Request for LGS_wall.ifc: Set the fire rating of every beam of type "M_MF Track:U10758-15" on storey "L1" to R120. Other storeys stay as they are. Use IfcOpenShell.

First a look at what the model holds.

```python
import ifcopenshell
import ifcopenshell.util.element

model = ifcopenshell.open("LGS_wall.ifc")
print(model.schema)
storey = next(s for s in model.by_type("IfcBuildingStorey") if s.Name == "L1")
beams = [e for e in ifcopenshell.util.element.get_decomposition(storey) if e.is_a("IfcBeam")]
seen = {}
for e in beams:
    element_type = ifcopenshell.util.element.get_type(e)
    key = (element_type.Name if element_type != e and element_type else None, ifcopenshell.util.element.get_pset(e, "Pset_BeamCommon", "FireRating"))
    seen[key] = seen.get(key, 0) + 1
for (name, value), count in sorted(seen.items(), key=str):
    print(count, "x", name, "|", value)
```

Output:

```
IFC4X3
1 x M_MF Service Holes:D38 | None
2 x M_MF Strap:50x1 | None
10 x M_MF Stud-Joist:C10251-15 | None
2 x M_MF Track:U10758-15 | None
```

```python
import ifcopenshell
import ifcopenshell.api.pset
import ifcopenshell.util.element

model = ifcopenshell.open("LGS_wall.ifc")

storey = next(s for s in model.by_type("IfcBuildingStorey") if s.Name == "L1")
beams = [e for e in ifcopenshell.util.element.get_decomposition(storey) if e.is_a("IfcBeam")]

count = 0
for e in beams:
    element_type = ifcopenshell.util.element.get_type(e)
    if element_type in (None, e) or element_type.Name != "M_MF Track:U10758-15":
        continue
    # add_pset returns the element's existing set when there is one.
    pset = ifcopenshell.api.pset.add_pset(model, product=e, name="Pset_BeamCommon")
    ifcopenshell.api.pset.edit_pset(model, pset=pset, properties={"FireRating": "R120"})
    count += 1

print(count, "beams updated")

model.write("LGS_wall_v2.ifc")
```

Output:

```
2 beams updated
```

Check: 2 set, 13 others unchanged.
